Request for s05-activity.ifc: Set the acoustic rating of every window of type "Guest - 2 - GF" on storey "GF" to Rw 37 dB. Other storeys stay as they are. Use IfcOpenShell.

First a look at what the model holds.

```python
import ifcopenshell
import ifcopenshell.util.element

model = ifcopenshell.open("s05-activity.ifc")
print(model.schema)
storey = next(s for s in model.by_type("IfcBuildingStorey") if s.Name == "GF")
windows = [e for e in ifcopenshell.util.element.get_decomposition(storey) if e.is_a("IfcWindow")]
seen = {}
for e in windows:
    element_type = ifcopenshell.util.element.get_type(e)
    key = (element_type.Name if element_type != e and element_type else None, ifcopenshell.util.element.get_pset(e, "Pset_WindowCommon", "AcousticRating"))
    seen[key] = seen.get(key, 0) + 1
for (name, value), count in sorted(seen.items(), key=str):
    print(count, "x", name, "|", value)
```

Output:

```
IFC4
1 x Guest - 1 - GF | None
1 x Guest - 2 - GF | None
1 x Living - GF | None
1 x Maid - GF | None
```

```python
import ifcopenshell
import ifcopenshell.api.pset
import ifcopenshell.util.element

model = ifcopenshell.open("s05-activity.ifc")

storey = next(s for s in model.by_type("IfcBuildingStorey") if s.Name == "GF")
windows = [e for e in ifcopenshell.util.element.get_decomposition(storey) if e.is_a("IfcWindow")]

count = 0
for e in windows:
    element_type = ifcopenshell.util.element.get_type(e)
    if element_type in (None, e) or element_type.Name != "Guest - 2 - GF":
        continue
    # add_pset returns the element's existing set when there is one.
    pset = ifcopenshell.api.pset.add_pset(model, product=e, name="Pset_WindowCommon")
    ifcopenshell.api.pset.edit_pset(model, pset=pset, properties={"AcousticRating": "Rw 37 dB"})
    count += 1

print(count, "windows updated")

model.write("s05-activity_updated.ifc")
```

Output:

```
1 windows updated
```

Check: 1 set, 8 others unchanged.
